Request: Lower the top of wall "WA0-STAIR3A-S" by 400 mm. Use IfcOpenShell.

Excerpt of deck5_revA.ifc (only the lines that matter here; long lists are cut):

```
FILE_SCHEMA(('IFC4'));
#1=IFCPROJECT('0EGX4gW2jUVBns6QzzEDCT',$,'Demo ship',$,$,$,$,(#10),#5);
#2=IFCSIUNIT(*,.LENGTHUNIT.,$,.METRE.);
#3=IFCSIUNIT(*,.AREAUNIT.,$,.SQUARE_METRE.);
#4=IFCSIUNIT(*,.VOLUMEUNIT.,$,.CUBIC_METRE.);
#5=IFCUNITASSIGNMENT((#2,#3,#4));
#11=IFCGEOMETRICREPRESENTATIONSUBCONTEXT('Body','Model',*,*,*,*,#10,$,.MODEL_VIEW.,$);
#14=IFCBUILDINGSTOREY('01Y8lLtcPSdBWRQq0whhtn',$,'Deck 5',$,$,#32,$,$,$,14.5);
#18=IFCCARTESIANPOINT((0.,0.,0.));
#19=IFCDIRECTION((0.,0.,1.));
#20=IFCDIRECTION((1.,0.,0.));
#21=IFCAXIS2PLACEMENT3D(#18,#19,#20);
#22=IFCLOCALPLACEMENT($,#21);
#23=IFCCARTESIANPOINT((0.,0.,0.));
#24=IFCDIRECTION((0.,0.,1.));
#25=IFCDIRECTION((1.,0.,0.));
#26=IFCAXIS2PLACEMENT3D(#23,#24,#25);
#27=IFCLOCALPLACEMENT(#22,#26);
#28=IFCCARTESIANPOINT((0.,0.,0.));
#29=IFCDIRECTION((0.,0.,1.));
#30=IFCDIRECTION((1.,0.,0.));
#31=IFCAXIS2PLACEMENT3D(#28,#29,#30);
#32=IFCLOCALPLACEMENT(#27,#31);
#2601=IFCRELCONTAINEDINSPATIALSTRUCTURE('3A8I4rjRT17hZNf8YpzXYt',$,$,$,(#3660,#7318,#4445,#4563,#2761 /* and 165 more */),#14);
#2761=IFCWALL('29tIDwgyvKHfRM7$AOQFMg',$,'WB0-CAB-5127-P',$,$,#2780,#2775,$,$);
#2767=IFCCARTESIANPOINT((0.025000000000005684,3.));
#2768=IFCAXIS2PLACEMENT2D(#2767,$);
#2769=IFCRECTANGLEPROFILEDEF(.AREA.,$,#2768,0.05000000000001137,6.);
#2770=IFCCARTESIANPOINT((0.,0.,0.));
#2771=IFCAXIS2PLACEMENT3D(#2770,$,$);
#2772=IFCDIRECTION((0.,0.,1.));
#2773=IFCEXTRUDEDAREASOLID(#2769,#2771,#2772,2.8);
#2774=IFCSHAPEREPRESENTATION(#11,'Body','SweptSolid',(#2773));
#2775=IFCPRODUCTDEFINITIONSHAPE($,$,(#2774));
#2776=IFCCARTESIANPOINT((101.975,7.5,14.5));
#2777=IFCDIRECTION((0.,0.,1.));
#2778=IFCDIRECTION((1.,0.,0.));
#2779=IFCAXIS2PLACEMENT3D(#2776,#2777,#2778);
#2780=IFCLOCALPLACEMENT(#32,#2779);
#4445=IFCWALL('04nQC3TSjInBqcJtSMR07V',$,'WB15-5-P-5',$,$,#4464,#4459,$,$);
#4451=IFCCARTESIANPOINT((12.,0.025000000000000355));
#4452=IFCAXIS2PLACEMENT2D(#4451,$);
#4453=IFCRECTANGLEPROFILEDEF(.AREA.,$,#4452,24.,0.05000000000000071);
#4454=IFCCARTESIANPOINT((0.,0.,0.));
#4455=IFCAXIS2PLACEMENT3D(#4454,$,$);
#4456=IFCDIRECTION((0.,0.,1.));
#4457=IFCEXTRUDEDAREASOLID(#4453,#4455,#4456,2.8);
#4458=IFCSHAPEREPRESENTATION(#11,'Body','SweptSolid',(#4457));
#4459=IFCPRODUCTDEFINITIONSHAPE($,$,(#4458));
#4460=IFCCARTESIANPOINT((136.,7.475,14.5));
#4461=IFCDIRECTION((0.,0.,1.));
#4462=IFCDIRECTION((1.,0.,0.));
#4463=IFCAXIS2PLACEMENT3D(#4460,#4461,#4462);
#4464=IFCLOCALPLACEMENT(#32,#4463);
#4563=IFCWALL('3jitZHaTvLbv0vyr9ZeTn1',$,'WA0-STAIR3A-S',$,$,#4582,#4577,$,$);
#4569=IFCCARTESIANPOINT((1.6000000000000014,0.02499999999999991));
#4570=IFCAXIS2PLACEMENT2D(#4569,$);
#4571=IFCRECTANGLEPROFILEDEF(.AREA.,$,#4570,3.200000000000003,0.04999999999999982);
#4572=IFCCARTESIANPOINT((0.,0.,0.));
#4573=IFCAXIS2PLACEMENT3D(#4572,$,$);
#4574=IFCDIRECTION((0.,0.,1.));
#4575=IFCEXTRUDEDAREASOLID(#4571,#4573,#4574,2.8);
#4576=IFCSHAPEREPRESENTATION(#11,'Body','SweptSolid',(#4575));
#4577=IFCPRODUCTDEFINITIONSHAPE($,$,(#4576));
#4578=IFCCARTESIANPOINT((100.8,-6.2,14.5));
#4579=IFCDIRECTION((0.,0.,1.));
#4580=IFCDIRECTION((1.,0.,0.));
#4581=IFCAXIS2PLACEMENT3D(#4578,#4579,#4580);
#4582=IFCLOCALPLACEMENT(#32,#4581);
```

```python
import ifcopenshell
import ifcopenshell.geom
import ifcopenshell.util.representation
import ifcopenshell.util.shape
import ifcopenshell.util.unit

model = ifcopenshell.open("deck5_revA.ifc")
unit_scale = ifcopenshell.util.unit.calculate_unit_scale(model)
settings = ifcopenshell.geom.settings()


def volume(element):
    """Net volume in cubic metres, openings subtracted."""
    shape = ifcopenshell.geom.create_shape(settings, element)
    return ifcopenshell.util.shape.get_volume(shape.geometry)


wall = model.by_guid("3jitZHaTvLbv0vyr9ZeTn1")
before = volume(wall)

body = ifcopenshell.util.representation.get_representation(wall, "Model", "Body")
solid = body.Items[0]
old_height = solid.Depth
solid.Depth -= 0.4 / unit_scale
after = volume(wall)

print(f"height {old_height:g} -> {solid.Depth:g}, volume {before:.3f} -> {after:.3f} m3")

model.write("deck5_revA_rev.ifc")
```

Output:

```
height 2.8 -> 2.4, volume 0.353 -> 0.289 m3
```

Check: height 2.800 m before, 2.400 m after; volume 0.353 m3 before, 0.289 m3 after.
